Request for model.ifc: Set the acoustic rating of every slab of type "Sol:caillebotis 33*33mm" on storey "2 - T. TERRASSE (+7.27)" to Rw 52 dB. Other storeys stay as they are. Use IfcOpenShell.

First a look at what the model holds.

```python
import ifcopenshell
import ifcopenshell.util.element

model = ifcopenshell.open("model.ifc")
print(model.schema)
storey = next(s for s in model.by_type("IfcBuildingStorey") if s.Name == "2 - T. TERRASSE (+7.27)")
slabs = [e for e in ifcopenshell.util.element.get_decomposition(storey) if e.is_a("IfcSlab")]
seen = {}
for e in slabs:
    element_type = ifcopenshell.util.element.get_type(e)
    key = (element_type.Name if element_type != e and element_type else None, ifcopenshell.util.element.get_pset(e, "Pset_SlabCommon", "AcousticRating"))
    seen[key] = seen.get(key, 0) + 1
for (name, value), count in sorted(seen.items(), key=str):
    print(count, "x", name, "|", value)
```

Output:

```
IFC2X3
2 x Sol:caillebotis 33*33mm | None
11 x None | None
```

```python
import ifcopenshell
import ifcopenshell.api.pset
import ifcopenshell.util.element

model = ifcopenshell.open("model.ifc")

storey = next(s for s in model.by_type("IfcBuildingStorey") if s.Name == "2 - T. TERRASSE (+7.27)")
slabs = [e for e in ifcopenshell.util.element.get_decomposition(storey) if e.is_a("IfcSlab")]

count = 0
for e in slabs:
    element_type = ifcopenshell.util.element.get_type(e)
    if element_type in (None, e) or element_type.Name != "Sol:caillebotis 33*33mm":
        continue
    # add_pset returns the element's existing set when there is one.
    pset = ifcopenshell.api.pset.add_pset(model, product=e, name="Pset_SlabCommon")
    ifcopenshell.api.pset.edit_pset(model, pset=pset, properties={"AcousticRating": "Rw 52 dB"})
    count += 1

print(count, "slabs updated")

model.write("model-out.ifc")
```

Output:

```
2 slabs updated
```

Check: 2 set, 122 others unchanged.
